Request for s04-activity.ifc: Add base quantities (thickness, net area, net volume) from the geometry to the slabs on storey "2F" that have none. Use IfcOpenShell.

First a look at what the model holds.

```python
import ifcopenshell
import ifcopenshell.util.element
import ifcopenshell.util.unit

model = ifcopenshell.open("s04-activity.ifc")
print(model.schema)
for unit_type in ("LENGTHUNIT", "AREAUNIT", "VOLUMEUNIT"):
    print(unit_type, ifcopenshell.util.unit.calculate_unit_scale(model, unit_type))
storey = next(s for s in model.by_type("IfcBuildingStorey") if s.Name == "2F")
slabs = [e for e in ifcopenshell.util.element.get_decomposition(storey) if e.is_a("IfcSlab")]
for e in sorted(slabs, key=lambda e: e.id()):
    print(e.id(), e.is_a(), e.Name, list(ifcopenshell.util.element.get_psets(e, qtos_only=True)), sep=" | ")
```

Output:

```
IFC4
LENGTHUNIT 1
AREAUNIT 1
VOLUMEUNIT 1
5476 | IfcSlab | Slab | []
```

```python
import ifcopenshell
import ifcopenshell.api.pset
import ifcopenshell.geom
import ifcopenshell.util.element
import ifcopenshell.util.shape
import ifcopenshell.util.unit

model = ifcopenshell.open("s04-activity.ifc")
unit_scale = ifcopenshell.util.unit.calculate_unit_scale(model)
area_scale = ifcopenshell.util.unit.calculate_unit_scale(model, "AREAUNIT")
volume_scale = ifcopenshell.util.unit.calculate_unit_scale(model, "VOLUMEUNIT")
settings = ifcopenshell.geom.settings()

storey = next(s for s in model.by_type("IfcBuildingStorey") if s.Name == "2F")
slabs = [e for e in ifcopenshell.util.element.get_decomposition(storey) if e.is_a("IfcSlab")]

for e in sorted(slabs, key=lambda e: e.id()):
    if ifcopenshell.util.element.get_psets(e, qtos_only=True, should_inherit=False):
        continue
    # Geometry comes back in metres, in the element's own axes.
    shape = ifcopenshell.geom.create_shape(settings, e)
    values = {
        "Width": ifcopenshell.util.shape.get_z(shape.geometry) / unit_scale,
        "NetArea": ifcopenshell.util.shape.get_footprint_area(shape.geometry) / area_scale,
        "NetVolume": ifcopenshell.util.shape.get_volume(shape.geometry) / volume_scale,
    }
    qto = ifcopenshell.api.pset.add_qto(model, product=e, name="Qto_SlabBaseQuantities")
    ifcopenshell.api.pset.edit_qto(model, qto=qto, properties=values)
    print(e.id(), {k: round(v, 3) for k, v in values.items()})

model.write("s04-activity_v2.ifc")
```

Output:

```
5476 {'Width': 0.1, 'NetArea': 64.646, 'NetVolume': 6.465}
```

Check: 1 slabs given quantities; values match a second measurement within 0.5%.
